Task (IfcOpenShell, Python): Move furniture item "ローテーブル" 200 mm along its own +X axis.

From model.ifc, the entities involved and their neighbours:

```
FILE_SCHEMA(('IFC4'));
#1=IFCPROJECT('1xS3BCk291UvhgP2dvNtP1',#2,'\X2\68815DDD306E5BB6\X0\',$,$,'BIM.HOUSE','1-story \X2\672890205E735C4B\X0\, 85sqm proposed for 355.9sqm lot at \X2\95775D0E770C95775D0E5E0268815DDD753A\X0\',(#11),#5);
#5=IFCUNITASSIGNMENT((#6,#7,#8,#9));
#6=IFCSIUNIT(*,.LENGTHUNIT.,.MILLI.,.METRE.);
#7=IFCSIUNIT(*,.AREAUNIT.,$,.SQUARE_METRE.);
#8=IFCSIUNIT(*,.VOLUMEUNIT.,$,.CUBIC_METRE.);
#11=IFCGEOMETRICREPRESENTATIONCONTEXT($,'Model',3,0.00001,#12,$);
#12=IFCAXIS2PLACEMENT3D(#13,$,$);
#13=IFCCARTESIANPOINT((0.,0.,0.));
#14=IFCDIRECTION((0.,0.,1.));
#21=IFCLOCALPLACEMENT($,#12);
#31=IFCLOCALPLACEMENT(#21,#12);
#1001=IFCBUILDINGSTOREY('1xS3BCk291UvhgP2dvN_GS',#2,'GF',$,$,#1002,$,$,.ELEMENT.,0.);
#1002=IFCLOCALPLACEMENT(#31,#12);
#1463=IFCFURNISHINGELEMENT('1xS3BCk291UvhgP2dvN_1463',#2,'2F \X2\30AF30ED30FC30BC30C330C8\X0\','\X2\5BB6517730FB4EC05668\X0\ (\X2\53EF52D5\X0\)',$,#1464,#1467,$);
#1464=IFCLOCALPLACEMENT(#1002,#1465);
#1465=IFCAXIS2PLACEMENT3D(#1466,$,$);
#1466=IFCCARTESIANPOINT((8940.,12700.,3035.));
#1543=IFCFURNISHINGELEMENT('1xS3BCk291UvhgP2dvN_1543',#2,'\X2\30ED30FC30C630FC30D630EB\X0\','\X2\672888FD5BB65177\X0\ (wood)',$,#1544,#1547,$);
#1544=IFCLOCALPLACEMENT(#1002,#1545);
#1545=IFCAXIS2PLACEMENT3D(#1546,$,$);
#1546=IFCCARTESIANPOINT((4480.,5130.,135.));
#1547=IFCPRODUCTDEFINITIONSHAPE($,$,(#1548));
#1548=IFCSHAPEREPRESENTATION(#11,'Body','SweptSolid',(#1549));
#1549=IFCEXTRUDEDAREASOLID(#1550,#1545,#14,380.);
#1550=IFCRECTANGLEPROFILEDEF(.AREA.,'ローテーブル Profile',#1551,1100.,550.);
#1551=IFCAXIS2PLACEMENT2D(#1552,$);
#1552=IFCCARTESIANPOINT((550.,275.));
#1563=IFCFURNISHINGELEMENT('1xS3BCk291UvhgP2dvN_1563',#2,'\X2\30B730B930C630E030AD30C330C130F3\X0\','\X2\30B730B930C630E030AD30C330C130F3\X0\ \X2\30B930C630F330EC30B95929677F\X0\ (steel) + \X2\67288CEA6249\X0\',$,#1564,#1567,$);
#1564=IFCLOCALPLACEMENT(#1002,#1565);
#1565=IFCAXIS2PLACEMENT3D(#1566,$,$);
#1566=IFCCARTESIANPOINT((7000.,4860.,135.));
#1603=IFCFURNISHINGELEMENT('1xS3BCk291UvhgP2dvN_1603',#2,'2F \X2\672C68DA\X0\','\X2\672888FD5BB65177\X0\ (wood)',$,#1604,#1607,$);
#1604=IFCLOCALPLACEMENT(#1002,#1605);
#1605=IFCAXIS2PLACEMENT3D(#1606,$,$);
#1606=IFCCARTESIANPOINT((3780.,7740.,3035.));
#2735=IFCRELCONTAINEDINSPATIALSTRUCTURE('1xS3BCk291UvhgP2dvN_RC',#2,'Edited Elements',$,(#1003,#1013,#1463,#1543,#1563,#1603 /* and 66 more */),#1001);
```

```python
import ifcopenshell
import ifcopenshell.api.geometry
import ifcopenshell.util.placement

model = ifcopenshell.open("model.ifc")

item = model.by_id(1543)
matrix = ifcopenshell.util.placement.get_local_placement(item.ObjectPlacement)
matrix[:3, 3] += matrix[:3, 0] * 200.0
ifcopenshell.api.geometry.edit_object_placement(model, product=item, matrix=matrix, is_si=False)

print(ifcopenshell.util.placement.get_local_placement(item.ObjectPlacement).round(3) + 0.0)

model.write("model_rev.ifc")
```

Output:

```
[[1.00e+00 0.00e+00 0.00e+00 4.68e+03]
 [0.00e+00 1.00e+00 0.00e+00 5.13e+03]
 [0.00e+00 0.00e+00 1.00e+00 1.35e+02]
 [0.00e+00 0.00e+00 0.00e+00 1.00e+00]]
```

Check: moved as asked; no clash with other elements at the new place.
